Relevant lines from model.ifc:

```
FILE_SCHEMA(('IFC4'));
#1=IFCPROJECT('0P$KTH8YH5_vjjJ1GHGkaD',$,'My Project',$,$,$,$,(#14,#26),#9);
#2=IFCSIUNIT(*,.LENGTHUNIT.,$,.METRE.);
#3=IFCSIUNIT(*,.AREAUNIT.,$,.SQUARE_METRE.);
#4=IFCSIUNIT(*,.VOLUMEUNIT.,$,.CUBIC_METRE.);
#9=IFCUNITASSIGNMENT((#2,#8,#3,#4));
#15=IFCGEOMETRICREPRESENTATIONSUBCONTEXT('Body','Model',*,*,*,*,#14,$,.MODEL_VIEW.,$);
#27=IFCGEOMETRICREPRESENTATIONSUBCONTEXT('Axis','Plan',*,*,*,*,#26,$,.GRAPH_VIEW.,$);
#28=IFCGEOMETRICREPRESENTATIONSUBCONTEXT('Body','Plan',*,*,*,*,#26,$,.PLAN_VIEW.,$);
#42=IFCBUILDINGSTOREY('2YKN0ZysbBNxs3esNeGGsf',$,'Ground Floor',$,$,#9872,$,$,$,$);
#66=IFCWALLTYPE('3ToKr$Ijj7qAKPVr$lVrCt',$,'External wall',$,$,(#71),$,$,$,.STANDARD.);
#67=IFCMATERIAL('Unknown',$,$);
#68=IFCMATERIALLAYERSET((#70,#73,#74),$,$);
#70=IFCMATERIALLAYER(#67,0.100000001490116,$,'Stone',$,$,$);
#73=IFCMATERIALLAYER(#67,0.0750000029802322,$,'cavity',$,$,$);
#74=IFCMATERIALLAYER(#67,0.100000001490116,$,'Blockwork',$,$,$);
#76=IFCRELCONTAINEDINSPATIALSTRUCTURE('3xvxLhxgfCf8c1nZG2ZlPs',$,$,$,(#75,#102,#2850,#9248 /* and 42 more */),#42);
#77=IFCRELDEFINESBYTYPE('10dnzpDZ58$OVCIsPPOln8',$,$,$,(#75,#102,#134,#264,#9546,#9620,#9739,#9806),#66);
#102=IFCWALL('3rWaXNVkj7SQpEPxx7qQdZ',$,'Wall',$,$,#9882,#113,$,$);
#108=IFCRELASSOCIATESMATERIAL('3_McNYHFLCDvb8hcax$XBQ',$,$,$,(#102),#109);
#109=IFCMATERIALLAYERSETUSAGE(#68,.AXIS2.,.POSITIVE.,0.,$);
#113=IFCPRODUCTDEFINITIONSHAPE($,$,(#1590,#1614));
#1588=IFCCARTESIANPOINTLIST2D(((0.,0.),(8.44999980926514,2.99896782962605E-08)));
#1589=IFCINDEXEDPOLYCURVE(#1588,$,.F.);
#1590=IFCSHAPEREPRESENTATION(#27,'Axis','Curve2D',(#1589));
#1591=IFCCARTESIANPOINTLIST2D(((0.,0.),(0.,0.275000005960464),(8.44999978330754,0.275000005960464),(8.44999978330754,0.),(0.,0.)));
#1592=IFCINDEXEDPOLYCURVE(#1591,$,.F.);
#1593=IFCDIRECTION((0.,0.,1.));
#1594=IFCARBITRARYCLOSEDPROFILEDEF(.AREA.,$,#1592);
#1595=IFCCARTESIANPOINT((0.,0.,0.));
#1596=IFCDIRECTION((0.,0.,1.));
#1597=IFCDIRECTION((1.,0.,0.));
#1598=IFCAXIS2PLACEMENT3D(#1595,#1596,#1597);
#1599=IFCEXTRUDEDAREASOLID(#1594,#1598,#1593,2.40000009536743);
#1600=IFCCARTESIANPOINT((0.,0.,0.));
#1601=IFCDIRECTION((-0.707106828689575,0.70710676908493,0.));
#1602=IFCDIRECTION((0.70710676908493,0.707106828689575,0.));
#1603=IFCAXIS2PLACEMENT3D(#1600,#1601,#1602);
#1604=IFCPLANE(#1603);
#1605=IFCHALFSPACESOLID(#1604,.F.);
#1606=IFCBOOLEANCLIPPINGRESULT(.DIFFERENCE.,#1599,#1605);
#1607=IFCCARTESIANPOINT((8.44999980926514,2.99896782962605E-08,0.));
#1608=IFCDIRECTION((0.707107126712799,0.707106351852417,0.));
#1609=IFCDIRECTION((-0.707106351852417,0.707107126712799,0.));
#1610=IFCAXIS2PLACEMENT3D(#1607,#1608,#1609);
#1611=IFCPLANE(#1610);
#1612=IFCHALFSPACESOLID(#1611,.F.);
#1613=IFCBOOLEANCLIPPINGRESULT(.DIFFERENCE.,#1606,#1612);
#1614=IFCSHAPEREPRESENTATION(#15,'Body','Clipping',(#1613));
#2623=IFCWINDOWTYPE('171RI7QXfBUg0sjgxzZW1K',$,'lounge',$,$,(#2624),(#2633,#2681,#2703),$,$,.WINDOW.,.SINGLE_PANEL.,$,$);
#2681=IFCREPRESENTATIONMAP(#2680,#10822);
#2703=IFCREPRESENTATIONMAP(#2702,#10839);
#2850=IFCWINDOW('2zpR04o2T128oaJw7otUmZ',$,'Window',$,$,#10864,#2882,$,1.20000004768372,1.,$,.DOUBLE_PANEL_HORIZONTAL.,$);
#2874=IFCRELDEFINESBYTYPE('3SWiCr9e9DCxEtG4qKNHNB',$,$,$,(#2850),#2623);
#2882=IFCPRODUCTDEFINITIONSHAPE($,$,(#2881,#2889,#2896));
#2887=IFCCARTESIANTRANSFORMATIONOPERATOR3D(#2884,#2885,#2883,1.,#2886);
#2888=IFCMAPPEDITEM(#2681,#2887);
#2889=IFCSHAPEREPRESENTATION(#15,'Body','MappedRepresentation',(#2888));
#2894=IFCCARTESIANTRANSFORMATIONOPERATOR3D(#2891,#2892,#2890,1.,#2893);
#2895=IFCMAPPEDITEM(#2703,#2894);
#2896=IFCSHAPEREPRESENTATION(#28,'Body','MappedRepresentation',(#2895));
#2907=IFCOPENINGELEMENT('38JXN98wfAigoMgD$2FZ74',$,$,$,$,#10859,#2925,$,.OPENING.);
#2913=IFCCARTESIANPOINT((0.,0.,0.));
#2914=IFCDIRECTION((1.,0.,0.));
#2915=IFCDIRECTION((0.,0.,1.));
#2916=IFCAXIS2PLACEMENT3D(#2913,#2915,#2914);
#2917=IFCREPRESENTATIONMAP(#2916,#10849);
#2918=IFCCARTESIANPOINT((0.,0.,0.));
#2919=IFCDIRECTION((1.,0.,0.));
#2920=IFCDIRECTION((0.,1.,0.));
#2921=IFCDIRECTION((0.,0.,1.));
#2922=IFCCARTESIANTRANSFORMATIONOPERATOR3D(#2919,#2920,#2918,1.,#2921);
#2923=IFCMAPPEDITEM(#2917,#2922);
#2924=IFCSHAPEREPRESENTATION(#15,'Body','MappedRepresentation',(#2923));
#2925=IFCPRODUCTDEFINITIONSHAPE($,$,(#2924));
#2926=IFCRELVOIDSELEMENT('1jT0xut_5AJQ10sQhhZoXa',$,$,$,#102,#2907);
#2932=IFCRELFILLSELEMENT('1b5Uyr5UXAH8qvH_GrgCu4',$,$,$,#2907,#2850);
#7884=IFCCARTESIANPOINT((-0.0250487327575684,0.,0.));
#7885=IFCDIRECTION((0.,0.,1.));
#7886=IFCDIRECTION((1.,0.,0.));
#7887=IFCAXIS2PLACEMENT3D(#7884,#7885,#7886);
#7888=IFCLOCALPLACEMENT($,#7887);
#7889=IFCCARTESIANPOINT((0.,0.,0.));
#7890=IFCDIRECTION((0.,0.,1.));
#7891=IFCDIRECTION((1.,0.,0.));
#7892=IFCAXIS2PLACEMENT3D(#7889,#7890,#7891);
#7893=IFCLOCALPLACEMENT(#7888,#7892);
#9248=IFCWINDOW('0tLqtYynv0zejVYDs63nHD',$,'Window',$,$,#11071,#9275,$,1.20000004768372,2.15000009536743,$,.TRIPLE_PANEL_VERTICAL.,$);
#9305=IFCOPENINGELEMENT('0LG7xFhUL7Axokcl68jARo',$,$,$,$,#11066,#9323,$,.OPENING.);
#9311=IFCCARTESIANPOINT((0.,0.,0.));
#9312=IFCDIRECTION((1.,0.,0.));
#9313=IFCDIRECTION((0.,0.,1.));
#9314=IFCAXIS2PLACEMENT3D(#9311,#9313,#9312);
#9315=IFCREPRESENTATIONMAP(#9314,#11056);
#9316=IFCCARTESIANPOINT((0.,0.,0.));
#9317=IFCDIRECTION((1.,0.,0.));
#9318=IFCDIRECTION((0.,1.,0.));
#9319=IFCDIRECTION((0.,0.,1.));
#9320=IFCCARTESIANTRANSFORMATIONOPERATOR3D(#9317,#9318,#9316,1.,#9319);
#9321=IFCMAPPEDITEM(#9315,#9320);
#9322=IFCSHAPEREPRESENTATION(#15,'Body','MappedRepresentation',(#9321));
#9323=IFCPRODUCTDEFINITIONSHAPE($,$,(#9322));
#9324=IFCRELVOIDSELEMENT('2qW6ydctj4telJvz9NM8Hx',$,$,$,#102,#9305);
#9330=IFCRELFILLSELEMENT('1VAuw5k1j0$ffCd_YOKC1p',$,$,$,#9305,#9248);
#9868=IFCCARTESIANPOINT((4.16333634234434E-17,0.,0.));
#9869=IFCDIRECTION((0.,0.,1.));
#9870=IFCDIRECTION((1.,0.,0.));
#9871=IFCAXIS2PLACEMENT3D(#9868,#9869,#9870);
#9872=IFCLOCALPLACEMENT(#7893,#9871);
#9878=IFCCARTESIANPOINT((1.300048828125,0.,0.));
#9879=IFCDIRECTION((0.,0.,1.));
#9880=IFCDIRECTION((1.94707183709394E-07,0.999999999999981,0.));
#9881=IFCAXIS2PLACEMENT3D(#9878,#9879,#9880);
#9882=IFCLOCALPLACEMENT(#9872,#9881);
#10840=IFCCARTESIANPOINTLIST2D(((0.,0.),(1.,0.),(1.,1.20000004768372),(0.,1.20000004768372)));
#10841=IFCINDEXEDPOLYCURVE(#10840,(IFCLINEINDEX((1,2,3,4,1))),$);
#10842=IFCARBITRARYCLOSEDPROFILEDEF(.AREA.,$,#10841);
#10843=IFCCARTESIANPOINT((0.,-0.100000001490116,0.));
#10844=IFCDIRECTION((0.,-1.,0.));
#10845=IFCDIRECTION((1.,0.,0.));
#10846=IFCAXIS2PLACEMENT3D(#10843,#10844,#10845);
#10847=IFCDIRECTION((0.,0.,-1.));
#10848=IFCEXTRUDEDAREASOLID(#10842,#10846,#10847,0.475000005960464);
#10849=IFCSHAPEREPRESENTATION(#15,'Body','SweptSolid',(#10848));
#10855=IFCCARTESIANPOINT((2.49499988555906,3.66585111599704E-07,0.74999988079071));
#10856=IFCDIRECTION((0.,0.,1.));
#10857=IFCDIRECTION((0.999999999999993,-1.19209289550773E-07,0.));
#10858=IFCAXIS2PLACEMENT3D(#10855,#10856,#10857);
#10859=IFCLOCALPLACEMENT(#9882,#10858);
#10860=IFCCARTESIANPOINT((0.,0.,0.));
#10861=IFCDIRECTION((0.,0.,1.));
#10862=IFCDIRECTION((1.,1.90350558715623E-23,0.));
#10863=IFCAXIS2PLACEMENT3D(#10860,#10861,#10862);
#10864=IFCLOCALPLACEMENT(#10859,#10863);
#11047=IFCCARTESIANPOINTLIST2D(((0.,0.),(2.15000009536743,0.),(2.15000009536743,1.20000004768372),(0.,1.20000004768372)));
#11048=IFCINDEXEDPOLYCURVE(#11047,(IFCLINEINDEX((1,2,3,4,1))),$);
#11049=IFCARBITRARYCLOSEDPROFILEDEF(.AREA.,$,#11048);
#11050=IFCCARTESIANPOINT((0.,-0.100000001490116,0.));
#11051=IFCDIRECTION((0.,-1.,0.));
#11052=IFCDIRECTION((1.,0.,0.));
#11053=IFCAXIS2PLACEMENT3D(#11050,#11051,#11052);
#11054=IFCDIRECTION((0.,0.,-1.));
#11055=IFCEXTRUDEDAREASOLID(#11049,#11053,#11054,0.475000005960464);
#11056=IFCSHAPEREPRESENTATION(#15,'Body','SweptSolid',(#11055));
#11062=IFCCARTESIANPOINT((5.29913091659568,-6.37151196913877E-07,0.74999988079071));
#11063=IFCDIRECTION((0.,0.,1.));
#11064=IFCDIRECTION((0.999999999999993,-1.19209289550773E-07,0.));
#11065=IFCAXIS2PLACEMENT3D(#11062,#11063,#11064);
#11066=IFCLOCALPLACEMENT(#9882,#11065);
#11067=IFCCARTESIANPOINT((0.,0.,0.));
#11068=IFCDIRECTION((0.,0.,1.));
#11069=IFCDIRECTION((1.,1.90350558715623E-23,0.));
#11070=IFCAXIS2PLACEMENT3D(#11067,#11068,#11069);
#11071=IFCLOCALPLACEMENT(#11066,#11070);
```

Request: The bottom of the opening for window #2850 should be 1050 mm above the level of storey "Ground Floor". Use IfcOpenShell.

```python
import numpy as np
import ifcopenshell
import ifcopenshell.api.geometry
import ifcopenshell.geom
import ifcopenshell.util.element
import ifcopenshell.util.placement
import ifcopenshell.util.shape
import ifcopenshell.util.unit

model = ifcopenshell.open("model.ifc")
unit_scale = ifcopenshell.util.unit.calculate_unit_scale(model)

window = model.by_guid("2zpR04o2T128oaJw7otUmZ")
opening = window.FillsVoids[0].RelatingOpeningElement
storey = ifcopenshell.util.element.get_container(window, ifc_class="IfcBuildingStorey")
level = ifcopenshell.util.placement.get_local_placement(storey.ObjectPlacement)[2, 3]

# The opening's origin need not be at the sill, so measure its lowest point.
shape = ifcopenshell.geom.create_shape(ifcopenshell.geom.settings(), opening)
bottom = ifcopenshell.util.shape.get_shape_bottom_elevation(shape, shape.geometry) / unit_scale
dz = level + 1.05 / unit_scale - bottom

shift = np.array([0.0, 0.0, dz])
# The window is placed relative to its opening, so it follows when the opening moves.
matrix = ifcopenshell.util.placement.get_local_placement(opening.ObjectPlacement)
matrix[:3, 3] += shift
ifcopenshell.api.geometry.edit_object_placement(
    model, product=opening, matrix=matrix, is_si=False, should_transform_children=True
)

print(f"moved by {dz * unit_scale:+.3f} m")

model.write("model-out.ifc")
```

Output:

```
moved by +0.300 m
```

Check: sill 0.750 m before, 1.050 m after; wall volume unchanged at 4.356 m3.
